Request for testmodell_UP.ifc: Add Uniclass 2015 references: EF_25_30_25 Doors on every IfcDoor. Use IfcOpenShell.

First a look at what the model holds.

```python
import ifcopenshell

model = ifcopenshell.open("testmodell_UP.ifc")
print(model.schema)
print("classifications:", [c.Name for c in model.by_type("IfcClassification")])
for ifc_class in ("IfcDoor", "IfcRoof", "IfcStair", "IfcWall", "IfcWindow"):
    print(ifc_class, len(model.by_type(ifc_class)))
```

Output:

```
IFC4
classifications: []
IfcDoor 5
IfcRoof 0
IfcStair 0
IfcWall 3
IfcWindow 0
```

```python
import ifcopenshell
import ifcopenshell.api.classification

model = ifcopenshell.open("testmodell_UP.ifc")

system = ifcopenshell.api.classification.add_classification(model, classification="Uniclass 2015")

codes = {
    "IfcDoor": ("EF_25_30_25", "Doors"),
}
for ifc_class, (code, name) in codes.items():
    products = model.by_type(ifc_class)
    ifcopenshell.api.classification.add_reference(
        model, products=products, classification=system, identification=code, name=name
    )
    print(code, len(products))

model.write("testmodell_UP_rev.ifc")
```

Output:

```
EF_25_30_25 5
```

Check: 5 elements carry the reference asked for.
